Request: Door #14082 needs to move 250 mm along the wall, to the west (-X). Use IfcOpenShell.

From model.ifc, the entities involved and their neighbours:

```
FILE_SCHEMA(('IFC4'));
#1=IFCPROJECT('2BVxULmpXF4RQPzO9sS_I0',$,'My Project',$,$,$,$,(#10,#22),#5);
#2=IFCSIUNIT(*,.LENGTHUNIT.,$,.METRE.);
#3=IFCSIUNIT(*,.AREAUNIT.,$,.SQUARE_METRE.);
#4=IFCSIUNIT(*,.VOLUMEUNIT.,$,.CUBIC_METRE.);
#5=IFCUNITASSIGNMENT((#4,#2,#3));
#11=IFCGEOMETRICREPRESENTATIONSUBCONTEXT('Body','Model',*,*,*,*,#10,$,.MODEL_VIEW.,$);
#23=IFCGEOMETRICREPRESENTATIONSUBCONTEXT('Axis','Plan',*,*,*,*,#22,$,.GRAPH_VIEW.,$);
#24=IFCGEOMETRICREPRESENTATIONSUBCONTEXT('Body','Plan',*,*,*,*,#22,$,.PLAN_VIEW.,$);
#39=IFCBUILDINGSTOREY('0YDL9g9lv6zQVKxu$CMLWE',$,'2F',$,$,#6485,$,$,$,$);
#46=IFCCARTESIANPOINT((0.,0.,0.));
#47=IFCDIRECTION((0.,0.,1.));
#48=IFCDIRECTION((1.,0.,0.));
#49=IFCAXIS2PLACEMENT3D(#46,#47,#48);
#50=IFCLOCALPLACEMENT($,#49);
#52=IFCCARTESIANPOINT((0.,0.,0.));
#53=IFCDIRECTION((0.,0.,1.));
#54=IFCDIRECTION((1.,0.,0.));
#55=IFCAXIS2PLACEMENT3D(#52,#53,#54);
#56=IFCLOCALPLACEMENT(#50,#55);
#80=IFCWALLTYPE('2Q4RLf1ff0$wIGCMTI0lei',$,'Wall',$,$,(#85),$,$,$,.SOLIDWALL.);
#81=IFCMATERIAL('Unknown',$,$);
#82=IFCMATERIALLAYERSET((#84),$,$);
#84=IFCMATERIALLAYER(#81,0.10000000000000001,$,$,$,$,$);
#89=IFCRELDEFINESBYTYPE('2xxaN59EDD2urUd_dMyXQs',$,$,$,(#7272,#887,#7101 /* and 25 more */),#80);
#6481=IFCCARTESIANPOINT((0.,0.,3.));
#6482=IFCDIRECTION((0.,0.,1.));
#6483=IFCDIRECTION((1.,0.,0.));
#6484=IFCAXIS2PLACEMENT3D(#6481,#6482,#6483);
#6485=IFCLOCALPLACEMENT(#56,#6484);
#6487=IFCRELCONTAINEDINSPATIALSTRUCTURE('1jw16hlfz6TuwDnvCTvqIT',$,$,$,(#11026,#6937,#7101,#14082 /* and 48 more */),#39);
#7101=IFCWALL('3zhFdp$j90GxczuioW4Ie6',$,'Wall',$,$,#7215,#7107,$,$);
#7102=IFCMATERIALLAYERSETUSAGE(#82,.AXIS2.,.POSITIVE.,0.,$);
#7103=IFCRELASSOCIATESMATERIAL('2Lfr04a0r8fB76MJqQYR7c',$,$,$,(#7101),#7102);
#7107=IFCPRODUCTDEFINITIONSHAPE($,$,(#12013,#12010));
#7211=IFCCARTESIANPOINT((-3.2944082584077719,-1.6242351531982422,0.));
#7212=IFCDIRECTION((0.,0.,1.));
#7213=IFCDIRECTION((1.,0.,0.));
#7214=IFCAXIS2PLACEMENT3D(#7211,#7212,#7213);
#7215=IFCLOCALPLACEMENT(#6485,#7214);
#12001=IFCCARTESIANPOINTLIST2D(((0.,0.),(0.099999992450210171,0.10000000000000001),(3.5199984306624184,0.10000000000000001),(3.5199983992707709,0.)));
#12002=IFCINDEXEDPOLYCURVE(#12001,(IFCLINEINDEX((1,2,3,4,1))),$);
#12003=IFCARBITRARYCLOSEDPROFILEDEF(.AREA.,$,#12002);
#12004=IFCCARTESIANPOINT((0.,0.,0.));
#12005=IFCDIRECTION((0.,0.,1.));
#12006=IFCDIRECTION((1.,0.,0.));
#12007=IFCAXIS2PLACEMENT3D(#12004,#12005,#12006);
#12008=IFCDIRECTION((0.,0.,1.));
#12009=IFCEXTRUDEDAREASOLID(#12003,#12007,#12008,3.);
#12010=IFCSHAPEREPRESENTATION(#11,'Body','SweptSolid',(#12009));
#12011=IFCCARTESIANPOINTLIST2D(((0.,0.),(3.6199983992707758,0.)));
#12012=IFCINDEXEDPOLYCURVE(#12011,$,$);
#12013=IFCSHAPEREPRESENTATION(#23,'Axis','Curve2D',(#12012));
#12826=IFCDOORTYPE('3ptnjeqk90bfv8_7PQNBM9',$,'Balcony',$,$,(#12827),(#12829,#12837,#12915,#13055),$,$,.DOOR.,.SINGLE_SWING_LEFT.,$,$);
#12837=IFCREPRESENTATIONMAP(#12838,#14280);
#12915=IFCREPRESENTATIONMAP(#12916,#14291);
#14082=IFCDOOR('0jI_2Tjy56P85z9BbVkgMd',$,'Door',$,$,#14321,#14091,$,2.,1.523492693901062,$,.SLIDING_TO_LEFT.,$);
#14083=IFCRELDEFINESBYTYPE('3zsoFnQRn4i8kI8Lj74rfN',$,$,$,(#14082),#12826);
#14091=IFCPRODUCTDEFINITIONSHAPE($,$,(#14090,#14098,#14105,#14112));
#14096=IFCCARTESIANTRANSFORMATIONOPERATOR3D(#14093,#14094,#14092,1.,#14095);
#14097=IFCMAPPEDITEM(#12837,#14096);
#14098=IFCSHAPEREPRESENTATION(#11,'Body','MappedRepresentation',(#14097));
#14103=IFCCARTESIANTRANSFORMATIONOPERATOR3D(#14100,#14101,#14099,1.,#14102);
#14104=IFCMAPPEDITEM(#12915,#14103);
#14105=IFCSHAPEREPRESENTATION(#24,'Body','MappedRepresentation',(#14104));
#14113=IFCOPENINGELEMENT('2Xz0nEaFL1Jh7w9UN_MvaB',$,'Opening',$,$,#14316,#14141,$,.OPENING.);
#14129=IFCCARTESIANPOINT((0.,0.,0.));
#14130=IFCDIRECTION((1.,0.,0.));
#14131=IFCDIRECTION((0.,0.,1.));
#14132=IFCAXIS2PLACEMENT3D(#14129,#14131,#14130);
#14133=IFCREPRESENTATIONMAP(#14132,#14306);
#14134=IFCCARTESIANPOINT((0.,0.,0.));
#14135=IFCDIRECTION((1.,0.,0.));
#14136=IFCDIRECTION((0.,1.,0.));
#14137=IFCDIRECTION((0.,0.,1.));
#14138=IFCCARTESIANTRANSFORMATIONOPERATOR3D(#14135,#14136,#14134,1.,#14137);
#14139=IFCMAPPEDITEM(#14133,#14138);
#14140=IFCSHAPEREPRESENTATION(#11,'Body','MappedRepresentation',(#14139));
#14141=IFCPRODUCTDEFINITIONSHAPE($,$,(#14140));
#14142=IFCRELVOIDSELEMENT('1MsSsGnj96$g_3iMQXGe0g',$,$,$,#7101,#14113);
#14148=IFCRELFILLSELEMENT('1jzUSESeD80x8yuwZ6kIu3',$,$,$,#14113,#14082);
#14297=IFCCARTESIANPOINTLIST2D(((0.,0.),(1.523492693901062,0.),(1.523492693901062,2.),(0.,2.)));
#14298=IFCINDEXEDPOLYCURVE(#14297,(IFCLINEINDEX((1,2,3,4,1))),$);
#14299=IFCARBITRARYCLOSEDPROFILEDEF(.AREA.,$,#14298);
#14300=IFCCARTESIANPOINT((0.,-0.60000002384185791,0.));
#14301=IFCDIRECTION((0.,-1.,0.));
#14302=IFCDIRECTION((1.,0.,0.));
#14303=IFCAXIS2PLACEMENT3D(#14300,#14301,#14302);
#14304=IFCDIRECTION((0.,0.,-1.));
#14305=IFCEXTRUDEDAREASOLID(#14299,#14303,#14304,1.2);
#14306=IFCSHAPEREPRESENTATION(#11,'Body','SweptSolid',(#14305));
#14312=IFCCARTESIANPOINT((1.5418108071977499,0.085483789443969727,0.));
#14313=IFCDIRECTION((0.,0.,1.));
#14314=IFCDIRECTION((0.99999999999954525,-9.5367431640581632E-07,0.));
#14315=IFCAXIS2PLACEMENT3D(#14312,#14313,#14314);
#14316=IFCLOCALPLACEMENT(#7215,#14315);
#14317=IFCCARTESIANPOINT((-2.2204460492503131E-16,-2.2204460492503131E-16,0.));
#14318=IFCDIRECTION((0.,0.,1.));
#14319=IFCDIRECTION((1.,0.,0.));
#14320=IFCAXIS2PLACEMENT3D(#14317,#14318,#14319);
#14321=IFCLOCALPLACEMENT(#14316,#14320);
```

```python
import ifcopenshell
import ifcopenshell.api.geometry
import ifcopenshell.util.placement

model = ifcopenshell.open("model.ifc")

door = model.by_guid("0jI_2Tjy56P85z9BbVkgMd")
opening = door.FillsVoids[0].RelatingOpeningElement
wall = opening.VoidsElements[0].RelatingBuildingElement

wall_matrix = ifcopenshell.util.placement.get_local_placement(wall.ObjectPlacement)
shift = wall_matrix[:3, 0] * -0.25
before = ifcopenshell.util.placement.get_local_placement(door.ObjectPlacement)[:3, 3].copy()

# The door is placed relative to its opening, so it follows when the opening moves.
matrix = ifcopenshell.util.placement.get_local_placement(opening.ObjectPlacement)
matrix[:3, 3] += shift
ifcopenshell.api.geometry.edit_object_placement(
    model, product=opening, matrix=matrix, is_si=False, should_transform_children=True
)

after = ifcopenshell.util.placement.get_local_placement(door.ObjectPlacement)[:3, 3]
print("door moved by", (after - before).round(3) + 0.0)

model.write("model_rev.ifc")
```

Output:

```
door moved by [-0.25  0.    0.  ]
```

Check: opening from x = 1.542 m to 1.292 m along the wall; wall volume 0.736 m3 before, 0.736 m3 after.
